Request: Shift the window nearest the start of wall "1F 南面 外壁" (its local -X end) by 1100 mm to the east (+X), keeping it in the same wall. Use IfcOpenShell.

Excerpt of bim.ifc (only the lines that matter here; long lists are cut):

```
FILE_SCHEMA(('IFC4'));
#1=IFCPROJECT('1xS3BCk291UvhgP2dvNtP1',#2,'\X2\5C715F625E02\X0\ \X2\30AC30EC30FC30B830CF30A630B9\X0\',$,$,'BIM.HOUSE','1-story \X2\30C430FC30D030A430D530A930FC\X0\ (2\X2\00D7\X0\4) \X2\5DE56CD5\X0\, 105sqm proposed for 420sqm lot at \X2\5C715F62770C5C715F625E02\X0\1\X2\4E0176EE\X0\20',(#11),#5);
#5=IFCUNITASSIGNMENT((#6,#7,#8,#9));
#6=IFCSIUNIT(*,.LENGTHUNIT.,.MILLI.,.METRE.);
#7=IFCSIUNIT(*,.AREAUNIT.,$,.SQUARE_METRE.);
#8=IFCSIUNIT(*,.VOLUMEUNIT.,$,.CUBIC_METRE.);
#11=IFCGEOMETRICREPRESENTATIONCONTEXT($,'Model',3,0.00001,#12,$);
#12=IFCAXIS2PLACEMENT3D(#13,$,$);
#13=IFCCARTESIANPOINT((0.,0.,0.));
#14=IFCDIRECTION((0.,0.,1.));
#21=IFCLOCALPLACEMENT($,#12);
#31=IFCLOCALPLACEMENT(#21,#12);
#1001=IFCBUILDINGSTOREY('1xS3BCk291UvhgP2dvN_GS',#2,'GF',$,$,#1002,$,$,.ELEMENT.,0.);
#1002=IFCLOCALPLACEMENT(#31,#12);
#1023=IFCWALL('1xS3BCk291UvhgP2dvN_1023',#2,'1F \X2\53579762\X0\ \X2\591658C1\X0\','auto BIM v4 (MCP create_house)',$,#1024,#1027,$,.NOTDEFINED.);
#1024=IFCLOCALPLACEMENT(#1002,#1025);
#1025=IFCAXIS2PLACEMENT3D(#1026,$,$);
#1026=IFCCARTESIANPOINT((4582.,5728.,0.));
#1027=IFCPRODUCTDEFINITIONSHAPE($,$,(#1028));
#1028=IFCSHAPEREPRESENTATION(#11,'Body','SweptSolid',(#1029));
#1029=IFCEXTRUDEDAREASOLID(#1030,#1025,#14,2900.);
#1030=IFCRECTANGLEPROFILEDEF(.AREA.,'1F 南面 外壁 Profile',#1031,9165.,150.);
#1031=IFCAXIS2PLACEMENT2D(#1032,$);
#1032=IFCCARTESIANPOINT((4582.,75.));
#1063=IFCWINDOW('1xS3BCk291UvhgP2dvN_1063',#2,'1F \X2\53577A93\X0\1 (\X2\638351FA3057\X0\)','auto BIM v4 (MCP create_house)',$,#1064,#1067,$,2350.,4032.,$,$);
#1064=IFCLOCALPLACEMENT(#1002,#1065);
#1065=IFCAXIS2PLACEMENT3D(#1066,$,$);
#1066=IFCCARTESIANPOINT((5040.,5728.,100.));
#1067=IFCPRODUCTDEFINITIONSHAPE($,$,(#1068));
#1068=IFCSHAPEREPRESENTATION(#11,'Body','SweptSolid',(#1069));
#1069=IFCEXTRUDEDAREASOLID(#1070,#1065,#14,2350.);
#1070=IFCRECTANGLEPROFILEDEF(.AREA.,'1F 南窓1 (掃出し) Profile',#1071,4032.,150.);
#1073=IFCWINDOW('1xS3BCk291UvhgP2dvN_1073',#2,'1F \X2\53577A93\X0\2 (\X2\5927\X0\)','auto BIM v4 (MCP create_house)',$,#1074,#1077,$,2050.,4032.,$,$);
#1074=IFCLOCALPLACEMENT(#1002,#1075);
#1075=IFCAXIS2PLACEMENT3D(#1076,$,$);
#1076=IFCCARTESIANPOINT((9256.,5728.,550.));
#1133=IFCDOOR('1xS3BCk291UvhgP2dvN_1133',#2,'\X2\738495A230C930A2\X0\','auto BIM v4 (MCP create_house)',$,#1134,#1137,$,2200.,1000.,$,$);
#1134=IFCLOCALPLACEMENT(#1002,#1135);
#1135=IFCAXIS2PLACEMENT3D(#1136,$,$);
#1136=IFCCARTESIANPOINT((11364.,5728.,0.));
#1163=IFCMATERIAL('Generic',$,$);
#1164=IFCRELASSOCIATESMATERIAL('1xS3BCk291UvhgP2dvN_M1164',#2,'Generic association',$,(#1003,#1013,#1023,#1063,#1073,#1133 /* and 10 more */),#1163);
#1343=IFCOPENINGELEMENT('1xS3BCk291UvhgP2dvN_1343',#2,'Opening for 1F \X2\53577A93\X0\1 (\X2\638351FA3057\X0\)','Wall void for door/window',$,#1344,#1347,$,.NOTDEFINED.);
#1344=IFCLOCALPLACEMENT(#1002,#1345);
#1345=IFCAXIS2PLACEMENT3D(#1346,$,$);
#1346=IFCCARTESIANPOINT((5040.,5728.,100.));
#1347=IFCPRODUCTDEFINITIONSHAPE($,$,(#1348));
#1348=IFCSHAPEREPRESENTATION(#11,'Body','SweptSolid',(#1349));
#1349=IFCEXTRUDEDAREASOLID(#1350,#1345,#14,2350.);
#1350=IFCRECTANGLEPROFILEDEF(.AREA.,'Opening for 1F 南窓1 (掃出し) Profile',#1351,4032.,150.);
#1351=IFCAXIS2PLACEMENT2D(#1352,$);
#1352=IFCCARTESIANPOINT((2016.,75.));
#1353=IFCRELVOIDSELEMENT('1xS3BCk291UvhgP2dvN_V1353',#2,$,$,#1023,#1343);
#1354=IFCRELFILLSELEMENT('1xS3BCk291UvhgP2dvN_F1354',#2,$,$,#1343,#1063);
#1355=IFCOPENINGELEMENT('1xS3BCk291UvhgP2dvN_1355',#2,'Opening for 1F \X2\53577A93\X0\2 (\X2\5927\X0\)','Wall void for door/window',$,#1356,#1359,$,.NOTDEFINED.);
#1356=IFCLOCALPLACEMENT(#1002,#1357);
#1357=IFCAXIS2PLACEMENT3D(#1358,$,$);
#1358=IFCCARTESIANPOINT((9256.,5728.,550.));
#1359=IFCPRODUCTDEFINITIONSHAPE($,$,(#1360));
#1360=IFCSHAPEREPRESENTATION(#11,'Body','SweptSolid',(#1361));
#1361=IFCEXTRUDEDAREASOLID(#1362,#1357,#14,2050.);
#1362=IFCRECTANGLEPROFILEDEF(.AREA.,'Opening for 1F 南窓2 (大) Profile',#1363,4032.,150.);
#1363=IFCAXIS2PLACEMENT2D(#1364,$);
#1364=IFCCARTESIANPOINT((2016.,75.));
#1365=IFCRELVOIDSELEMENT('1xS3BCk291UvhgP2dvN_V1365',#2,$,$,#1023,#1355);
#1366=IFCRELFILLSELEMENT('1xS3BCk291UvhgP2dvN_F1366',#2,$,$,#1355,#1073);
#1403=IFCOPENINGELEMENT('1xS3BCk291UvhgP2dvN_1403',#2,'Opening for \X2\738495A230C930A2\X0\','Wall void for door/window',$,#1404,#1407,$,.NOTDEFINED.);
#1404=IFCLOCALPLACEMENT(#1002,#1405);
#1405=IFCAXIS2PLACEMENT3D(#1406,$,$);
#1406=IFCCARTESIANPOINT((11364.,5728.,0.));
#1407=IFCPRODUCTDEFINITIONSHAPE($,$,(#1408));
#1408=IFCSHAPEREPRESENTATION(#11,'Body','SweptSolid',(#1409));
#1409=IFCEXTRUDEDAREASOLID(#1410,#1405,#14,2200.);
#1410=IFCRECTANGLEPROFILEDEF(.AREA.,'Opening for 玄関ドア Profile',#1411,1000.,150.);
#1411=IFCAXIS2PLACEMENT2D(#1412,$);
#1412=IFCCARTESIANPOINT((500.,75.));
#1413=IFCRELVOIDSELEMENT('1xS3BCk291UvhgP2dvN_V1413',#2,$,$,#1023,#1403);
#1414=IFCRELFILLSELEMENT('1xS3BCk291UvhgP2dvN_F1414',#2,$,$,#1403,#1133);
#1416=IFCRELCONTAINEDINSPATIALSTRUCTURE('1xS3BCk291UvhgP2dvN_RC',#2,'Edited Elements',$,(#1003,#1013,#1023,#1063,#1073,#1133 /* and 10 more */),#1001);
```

```python
import ifcopenshell
import ifcopenshell.api.geometry
import ifcopenshell.util.placement
import ifcopenshell.util.unit

model = ifcopenshell.open("bim.ifc")
unit_scale = ifcopenshell.util.unit.calculate_unit_scale(model)

window = model.by_guid("1xS3BCk291UvhgP2dvN_1063")
opening = window.FillsVoids[0].RelatingOpeningElement
wall = opening.VoidsElements[0].RelatingBuildingElement

wall_matrix = ifcopenshell.util.placement.get_local_placement(wall.ObjectPlacement)
shift = wall_matrix[:3, 0] * 1.1 / unit_scale
before = ifcopenshell.util.placement.get_local_placement(window.ObjectPlacement)[:3, 3].copy()

# The window is not placed relative to its opening, so move both.
for product in (opening, window):
    matrix = ifcopenshell.util.placement.get_local_placement(product.ObjectPlacement)
    matrix[:3, 3] += shift
    ifcopenshell.api.geometry.edit_object_placement(model, product=product, matrix=matrix, is_si=False)

after = ifcopenshell.util.placement.get_local_placement(window.ObjectPlacement)[:3, 3]
print("window moved by", (after - before).round(3) + 0.0)

model.write("bim_rev.ifc")
```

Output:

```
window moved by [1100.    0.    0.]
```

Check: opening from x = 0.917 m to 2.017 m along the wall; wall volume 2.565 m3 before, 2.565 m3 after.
